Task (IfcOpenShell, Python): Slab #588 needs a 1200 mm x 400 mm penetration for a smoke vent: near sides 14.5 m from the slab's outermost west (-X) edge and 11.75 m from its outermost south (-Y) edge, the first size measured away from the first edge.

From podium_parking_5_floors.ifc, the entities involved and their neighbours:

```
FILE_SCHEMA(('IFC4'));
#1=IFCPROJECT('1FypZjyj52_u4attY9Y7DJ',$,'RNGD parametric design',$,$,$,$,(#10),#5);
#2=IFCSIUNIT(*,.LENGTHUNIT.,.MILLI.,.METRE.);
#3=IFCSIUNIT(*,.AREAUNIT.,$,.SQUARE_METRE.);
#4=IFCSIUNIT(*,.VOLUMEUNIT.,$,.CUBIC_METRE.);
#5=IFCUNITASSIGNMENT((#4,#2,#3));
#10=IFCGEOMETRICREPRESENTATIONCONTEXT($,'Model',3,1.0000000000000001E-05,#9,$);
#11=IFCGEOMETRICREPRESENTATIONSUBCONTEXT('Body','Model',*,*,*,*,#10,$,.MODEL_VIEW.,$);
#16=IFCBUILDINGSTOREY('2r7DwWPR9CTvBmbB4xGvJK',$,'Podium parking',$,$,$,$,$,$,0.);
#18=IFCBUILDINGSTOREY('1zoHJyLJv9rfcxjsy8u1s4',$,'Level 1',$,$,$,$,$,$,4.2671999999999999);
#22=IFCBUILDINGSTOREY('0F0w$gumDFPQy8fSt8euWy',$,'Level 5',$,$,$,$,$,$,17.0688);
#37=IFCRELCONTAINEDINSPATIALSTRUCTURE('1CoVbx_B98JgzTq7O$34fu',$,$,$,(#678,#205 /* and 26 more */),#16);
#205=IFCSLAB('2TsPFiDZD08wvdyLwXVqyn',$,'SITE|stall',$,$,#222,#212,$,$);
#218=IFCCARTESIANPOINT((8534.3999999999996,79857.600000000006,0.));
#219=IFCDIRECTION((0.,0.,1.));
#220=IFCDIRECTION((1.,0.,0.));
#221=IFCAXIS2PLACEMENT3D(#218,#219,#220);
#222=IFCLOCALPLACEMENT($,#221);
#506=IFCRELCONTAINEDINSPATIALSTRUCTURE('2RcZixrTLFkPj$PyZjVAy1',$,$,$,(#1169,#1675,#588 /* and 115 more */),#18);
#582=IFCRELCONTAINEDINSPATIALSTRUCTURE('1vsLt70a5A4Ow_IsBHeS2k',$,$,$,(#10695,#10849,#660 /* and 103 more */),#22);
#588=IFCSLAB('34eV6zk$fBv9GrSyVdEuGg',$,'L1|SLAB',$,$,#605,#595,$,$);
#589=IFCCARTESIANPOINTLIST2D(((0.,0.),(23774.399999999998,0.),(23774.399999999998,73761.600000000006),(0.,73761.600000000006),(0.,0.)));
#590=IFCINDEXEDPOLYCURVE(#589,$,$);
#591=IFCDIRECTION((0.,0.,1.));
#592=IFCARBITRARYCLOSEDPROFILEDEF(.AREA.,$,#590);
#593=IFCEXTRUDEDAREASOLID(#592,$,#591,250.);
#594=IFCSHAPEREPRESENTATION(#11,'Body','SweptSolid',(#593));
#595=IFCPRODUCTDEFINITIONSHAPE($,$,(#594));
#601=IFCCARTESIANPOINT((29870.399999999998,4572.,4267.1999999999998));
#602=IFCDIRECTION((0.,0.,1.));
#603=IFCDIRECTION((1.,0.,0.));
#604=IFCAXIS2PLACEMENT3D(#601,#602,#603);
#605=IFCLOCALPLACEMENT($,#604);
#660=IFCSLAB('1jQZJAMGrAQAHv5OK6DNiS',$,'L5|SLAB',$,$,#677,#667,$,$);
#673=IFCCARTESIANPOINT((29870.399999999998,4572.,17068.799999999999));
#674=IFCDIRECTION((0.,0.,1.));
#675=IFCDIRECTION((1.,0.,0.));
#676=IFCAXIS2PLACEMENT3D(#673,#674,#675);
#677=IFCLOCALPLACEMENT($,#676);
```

```python
import numpy as np
import ifcopenshell
import ifcopenshell.api.feature
import ifcopenshell.api.geometry
import ifcopenshell.api.root
import ifcopenshell.geom
import ifcopenshell.util.placement
import ifcopenshell.util.representation
import ifcopenshell.util.shape
import ifcopenshell.util.unit

model = ifcopenshell.open("podium_parking_5_floors.ifc")
unit_scale = ifcopenshell.util.unit.calculate_unit_scale(model)
settings = ifcopenshell.geom.settings()


def volume(element):
    """Net volume in cubic metres, openings subtracted."""
    shape = ifcopenshell.geom.create_shape(settings, element)
    return ifcopenshell.util.shape.get_volume(shape.geometry)


slab = model.by_id(588)
before = volume(slab)

# Extent in the slab's own axes, in metres. The edges named are its -X and -Y sides.
slab_shape = ifcopenshell.geom.create_shape(settings, slab)
vertices = ifcopenshell.util.shape.get_vertices(slab_shape.geometry)
x_min, y_min, bottom = vertices.min(axis=0)
top = vertices[:, 2].max()

opening = ifcopenshell.api.root.create_entity(model, ifc_class="IfcOpeningElement", name="Smoke vent opening", predefined_type="OPENING")
context = ifcopenshell.util.representation.get_context(model, "Model", "Body", "MODEL_VIEW")
width, depth = 1.2, 0.4
outline = [(0.0, 0.0), (width, 0.0), (width, depth), (0.0, depth), (0.0, 0.0)]
# Overshoot both faces by 50 mm so the cut is clean.
shape = ifcopenshell.api.geometry.add_slab_representation(
    model, context=context, depth=top - bottom + 0.1, polyline=outline
)
ifcopenshell.api.geometry.assign_representation(model, product=opening, representation=shape)

matrix = ifcopenshell.util.placement.get_local_placement(slab.ObjectPlacement)
matrix[:, 3] = matrix @ np.append(np.array([x_min + 14.5, y_min + 11.75, bottom - 0.05]) / unit_scale, 1.0)
ifcopenshell.api.geometry.edit_object_placement(model, product=opening, matrix=matrix, is_si=False)
ifcopenshell.api.feature.add_feature(model, feature=opening, element=slab)

after = volume(slab)

print(f"slab volume {before:.3f} -> {after:.3f} m3")

model.write("podium_parking_5_floors_updated.ifc")
```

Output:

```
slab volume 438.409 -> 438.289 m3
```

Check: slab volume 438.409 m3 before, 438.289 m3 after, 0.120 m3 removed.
